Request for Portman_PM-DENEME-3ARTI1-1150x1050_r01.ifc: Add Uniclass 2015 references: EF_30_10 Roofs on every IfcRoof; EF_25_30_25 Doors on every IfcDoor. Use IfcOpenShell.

First a look at what the model holds.

```python
import ifcopenshell

model = ifcopenshell.open("Portman_PM-DENEME-3ARTI1-1150x1050_r01.ifc")
print(model.schema)
print("classifications:", [c.Name for c in model.by_type("IfcClassification")])
for ifc_class in ("IfcDoor", "IfcRoof", "IfcStair", "IfcWall", "IfcWindow"):
    print(ifc_class, len(model.by_type(ifc_class)))
```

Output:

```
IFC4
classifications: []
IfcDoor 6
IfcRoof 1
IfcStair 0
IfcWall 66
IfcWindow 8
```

```python
import ifcopenshell
import ifcopenshell.api.classification

model = ifcopenshell.open("Portman_PM-DENEME-3ARTI1-1150x1050_r01.ifc")

system = ifcopenshell.api.classification.add_classification(model, classification="Uniclass 2015")

codes = {
    "IfcRoof": ("EF_30_10", "Roofs"),
    "IfcDoor": ("EF_25_30_25", "Doors"),
}
for ifc_class, (code, name) in codes.items():
    products = model.by_type(ifc_class)
    ifcopenshell.api.classification.add_reference(
        model, products=products, classification=system, identification=code, name=name
    )
    print(code, len(products))

model.write("Portman_PM-DENEME-3ARTI1-1150x1050_r01-out.ifc")
```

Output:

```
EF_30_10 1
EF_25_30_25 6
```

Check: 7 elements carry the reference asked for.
